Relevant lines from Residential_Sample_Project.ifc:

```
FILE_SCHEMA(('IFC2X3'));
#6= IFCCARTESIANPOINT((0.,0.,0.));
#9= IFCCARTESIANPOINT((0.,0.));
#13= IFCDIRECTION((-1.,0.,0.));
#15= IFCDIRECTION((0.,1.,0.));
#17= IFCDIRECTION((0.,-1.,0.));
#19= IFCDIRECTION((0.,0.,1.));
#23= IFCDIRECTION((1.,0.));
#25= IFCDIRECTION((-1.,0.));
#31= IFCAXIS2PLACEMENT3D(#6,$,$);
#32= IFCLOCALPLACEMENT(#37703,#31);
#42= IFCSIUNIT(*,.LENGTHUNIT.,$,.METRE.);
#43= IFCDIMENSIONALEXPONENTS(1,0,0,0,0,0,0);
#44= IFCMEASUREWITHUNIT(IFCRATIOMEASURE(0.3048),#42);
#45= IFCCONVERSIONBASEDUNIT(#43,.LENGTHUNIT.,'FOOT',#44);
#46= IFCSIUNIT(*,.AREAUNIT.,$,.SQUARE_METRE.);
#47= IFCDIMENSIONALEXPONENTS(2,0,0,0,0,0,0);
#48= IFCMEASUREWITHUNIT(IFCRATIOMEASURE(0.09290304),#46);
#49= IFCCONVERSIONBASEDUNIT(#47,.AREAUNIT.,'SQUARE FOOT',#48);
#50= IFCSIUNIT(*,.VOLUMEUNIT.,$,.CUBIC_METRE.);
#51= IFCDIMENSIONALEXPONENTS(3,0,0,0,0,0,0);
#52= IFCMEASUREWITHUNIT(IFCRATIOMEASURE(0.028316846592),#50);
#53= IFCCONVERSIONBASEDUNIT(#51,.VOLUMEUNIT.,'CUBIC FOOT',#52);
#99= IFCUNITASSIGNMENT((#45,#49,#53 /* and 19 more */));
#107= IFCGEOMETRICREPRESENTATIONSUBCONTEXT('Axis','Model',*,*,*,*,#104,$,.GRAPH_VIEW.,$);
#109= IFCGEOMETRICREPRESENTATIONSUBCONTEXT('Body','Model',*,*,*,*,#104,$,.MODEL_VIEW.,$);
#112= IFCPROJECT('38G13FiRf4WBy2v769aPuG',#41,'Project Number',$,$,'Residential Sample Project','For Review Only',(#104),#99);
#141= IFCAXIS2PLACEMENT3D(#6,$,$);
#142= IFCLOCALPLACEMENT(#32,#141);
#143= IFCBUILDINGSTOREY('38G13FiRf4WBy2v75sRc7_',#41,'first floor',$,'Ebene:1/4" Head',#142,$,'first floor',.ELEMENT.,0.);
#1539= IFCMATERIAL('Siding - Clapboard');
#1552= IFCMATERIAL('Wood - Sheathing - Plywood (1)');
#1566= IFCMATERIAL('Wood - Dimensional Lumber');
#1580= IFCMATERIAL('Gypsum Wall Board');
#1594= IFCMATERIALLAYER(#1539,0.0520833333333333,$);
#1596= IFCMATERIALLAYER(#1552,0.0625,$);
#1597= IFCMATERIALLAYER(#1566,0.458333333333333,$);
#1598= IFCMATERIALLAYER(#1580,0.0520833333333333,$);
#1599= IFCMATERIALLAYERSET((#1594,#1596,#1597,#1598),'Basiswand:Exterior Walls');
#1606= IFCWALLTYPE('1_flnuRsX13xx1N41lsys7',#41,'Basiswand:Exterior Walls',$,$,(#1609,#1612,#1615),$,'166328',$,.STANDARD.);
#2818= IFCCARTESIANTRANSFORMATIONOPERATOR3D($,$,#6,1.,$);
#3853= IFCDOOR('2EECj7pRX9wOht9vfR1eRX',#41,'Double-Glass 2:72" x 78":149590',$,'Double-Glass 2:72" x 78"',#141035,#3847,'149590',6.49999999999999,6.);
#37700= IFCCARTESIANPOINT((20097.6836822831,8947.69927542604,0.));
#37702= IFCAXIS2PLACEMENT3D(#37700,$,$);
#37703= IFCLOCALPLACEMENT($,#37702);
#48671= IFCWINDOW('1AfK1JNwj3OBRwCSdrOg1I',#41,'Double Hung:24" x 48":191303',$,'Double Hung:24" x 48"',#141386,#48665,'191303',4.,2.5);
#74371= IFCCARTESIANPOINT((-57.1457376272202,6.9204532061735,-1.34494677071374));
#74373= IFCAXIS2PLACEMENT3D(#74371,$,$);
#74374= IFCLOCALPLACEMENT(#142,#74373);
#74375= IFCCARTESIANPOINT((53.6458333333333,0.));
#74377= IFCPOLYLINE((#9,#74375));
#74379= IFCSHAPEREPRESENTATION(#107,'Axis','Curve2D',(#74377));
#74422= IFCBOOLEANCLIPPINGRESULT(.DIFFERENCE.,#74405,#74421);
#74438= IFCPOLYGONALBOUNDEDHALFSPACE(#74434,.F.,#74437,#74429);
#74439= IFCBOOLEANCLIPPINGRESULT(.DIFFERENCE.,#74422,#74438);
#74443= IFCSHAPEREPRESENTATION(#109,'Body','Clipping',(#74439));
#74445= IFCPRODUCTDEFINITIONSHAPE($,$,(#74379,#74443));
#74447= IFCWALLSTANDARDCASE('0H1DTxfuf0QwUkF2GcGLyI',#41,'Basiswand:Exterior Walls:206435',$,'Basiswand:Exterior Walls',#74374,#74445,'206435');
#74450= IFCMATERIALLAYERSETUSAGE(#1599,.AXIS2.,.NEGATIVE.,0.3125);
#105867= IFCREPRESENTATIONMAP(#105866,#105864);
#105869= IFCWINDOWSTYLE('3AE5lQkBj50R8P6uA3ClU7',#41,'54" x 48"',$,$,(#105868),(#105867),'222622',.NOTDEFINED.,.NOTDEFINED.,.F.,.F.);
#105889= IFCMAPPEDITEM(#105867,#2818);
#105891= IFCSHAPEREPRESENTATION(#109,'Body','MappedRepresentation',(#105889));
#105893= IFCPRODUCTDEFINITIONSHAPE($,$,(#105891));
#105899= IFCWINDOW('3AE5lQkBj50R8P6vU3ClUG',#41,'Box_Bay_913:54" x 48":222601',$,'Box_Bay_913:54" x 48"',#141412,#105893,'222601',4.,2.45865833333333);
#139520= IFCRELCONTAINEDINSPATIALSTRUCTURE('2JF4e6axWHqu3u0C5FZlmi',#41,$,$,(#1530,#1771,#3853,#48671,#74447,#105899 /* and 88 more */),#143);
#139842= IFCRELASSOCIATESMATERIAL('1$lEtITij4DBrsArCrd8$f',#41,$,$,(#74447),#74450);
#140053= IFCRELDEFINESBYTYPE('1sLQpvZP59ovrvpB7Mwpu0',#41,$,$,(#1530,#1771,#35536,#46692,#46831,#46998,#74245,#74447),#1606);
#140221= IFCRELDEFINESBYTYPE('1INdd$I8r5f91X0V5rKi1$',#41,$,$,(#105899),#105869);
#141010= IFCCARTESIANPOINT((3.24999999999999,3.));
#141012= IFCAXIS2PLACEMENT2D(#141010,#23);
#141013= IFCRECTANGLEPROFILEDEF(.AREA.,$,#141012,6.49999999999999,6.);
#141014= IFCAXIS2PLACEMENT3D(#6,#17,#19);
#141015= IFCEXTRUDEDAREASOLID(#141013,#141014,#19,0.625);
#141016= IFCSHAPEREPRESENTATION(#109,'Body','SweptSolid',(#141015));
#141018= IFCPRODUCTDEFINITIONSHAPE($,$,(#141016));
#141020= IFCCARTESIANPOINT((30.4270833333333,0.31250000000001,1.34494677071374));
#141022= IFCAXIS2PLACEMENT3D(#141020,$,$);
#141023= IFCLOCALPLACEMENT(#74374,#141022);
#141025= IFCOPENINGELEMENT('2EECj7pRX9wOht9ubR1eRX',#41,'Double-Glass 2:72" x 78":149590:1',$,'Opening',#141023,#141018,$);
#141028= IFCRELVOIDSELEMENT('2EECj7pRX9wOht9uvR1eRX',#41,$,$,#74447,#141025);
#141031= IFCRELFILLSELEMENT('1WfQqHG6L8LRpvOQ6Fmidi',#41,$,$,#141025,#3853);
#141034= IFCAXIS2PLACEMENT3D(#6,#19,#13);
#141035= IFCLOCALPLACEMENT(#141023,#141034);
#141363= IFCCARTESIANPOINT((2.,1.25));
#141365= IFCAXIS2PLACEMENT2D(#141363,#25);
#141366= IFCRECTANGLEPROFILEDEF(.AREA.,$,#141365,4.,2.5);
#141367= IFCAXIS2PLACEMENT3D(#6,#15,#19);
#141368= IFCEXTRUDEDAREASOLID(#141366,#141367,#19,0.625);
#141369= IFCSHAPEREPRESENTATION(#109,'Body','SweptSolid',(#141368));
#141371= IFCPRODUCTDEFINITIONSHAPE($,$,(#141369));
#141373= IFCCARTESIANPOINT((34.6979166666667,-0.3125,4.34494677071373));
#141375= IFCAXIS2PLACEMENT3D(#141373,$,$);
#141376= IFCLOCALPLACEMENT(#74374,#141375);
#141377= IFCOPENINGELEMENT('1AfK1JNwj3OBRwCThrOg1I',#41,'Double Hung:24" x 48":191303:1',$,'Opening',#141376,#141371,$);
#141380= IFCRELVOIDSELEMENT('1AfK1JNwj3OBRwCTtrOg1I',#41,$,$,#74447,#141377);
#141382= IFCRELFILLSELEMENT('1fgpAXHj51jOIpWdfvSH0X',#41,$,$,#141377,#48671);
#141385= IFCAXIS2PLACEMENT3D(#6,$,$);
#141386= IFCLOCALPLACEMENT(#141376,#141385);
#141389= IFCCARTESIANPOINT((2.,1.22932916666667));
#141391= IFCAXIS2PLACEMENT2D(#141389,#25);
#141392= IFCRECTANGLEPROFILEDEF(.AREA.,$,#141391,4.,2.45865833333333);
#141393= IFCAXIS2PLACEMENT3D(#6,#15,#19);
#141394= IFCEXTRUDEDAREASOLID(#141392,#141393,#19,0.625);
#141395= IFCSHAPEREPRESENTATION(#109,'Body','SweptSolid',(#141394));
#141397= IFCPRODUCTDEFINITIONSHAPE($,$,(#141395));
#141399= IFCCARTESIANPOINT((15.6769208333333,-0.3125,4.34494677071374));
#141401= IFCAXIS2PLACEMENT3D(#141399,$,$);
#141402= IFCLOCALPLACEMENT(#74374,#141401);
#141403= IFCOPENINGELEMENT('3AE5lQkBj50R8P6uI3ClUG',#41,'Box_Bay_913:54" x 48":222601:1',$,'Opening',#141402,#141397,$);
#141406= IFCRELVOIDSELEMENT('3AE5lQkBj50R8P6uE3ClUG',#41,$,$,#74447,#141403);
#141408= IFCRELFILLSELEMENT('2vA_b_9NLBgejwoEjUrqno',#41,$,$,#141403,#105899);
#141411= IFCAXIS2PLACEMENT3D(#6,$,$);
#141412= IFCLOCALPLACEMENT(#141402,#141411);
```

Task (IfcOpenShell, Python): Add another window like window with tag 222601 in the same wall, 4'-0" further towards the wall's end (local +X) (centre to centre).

```python
import ifcopenshell
import ifcopenshell.api.feature
import ifcopenshell.api.geometry
import ifcopenshell.api.root
import ifcopenshell.geom
import ifcopenshell.util.element
import ifcopenshell.util.placement
import ifcopenshell.util.shape
import ifcopenshell.util.unit

model = ifcopenshell.open("Residential_Sample_Project.ifc")
unit_scale = ifcopenshell.util.unit.calculate_unit_scale(model)
settings = ifcopenshell.geom.settings()


def volume(element):
    """Net volume in cubic metres, openings subtracted."""
    shape = ifcopenshell.geom.create_shape(settings, element)
    return ifcopenshell.util.shape.get_volume(shape.geometry)


def reuse_history(source, copy):
    """copy_class also copies each property set's owner history, people and application; keep the originals."""
    for rel in copy.IsDefinedBy:
        if rel.is_a("IfcRelDefinesByProperties") and (history := rel.RelatingPropertyDefinition.OwnerHistory):
            rel.RelatingPropertyDefinition.OwnerHistory = source.OwnerHistory
            ifcopenshell.util.element.remove_deep2(model, history)


window = model.by_id(105899)
opening = window.FillsVoids[0].RelatingOpeningElement
wall = opening.VoidsElements[0].RelatingBuildingElement
before = volume(wall)
shift = ifcopenshell.util.placement.get_local_placement(wall.ObjectPlacement)[:3, 0] * 48 * 0.0254 / unit_scale

# copy_class copies the void relationship, type, container and properties, but no geometry.
new_opening = ifcopenshell.api.root.copy_class(model, product=opening)
new_opening.Representation = ifcopenshell.util.element.copy_deep(
    model, opening.Representation, exclude=["IfcGeometricRepresentationContext", "IfcRepresentationMap"]
)
new_opening.Name = 'Box_Bay_913:54" x 48"'
new_window = ifcopenshell.api.root.copy_class(model, product=window)
new_window.Representation = ifcopenshell.util.element.copy_deep(
    model, window.Representation, exclude=["IfcGeometricRepresentationContext", "IfcRepresentationMap"]
)
new_window.Name = 'Box_Bay_913:54" x 48"'
new_window.Tag = None
reuse_history(window, new_window)
fills = ifcopenshell.api.feature.add_filling(model, opening=new_opening, element=new_window)
fills.OwnerHistory = new_window.OwnerHistory  # required in IFC2X3

for old, new in ((opening, new_opening), (window, new_window)):
    matrix = ifcopenshell.util.placement.get_local_placement(old.ObjectPlacement)
    matrix[:3, 3] += shift
    ifcopenshell.api.geometry.edit_object_placement(model, product=new, matrix=matrix, is_si=False)

after = volume(wall)

print(f"wall volume {before:.3f} -> {after:.3f} m3")

model.write("Residential_Sample_Project_v2.ifc")
```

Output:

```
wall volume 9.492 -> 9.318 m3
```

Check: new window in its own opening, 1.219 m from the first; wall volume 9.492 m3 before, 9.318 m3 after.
